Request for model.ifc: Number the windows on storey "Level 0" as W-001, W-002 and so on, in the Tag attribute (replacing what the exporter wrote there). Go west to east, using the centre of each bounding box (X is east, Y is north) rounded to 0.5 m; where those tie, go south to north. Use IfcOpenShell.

First a look at what the model holds.

```python
import ifcopenshell
import ifcopenshell.util.element
import ifcopenshell.util.placement

model = ifcopenshell.open("model.ifc")
print(model.schema)
storey = next(s for s in model.by_type("IfcBuildingStorey") if s.Name == "Level 0")
windows = [e for e in ifcopenshell.util.element.get_decomposition(storey) if e.is_a("IfcWindow")]
for e in sorted(windows, key=lambda e: e.id()):
    origin = ifcopenshell.util.placement.get_local_placement(e.ObjectPlacement)[:3, 3]
    print(e.id(), e.Tag, e.Name, origin.round(2) + 0.0, sep=" | ")
```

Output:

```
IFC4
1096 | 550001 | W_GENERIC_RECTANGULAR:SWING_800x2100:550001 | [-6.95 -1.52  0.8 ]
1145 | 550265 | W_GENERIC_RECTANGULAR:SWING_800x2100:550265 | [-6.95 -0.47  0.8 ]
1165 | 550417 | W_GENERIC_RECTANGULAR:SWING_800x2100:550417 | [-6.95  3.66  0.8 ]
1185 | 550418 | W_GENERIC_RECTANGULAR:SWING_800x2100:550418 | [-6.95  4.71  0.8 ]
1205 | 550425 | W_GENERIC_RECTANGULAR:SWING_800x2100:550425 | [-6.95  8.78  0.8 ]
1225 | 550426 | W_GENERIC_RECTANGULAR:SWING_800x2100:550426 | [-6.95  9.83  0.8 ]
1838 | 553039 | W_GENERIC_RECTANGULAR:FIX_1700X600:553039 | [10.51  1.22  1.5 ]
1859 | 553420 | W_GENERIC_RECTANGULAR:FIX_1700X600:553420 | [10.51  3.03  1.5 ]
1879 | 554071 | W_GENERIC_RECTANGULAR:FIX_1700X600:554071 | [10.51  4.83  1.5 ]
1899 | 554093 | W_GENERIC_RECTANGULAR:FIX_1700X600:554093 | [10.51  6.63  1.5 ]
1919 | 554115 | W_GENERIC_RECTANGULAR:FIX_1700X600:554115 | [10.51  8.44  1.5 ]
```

```python
import ifcopenshell
import ifcopenshell.geom
import ifcopenshell.util.element
import ifcopenshell.util.shape

model = ifcopenshell.open("model.ifc")
settings = ifcopenshell.geom.settings()
settings.set("use-world-coords", True)


def centre(element):
    shape = ifcopenshell.geom.create_shape(settings, element)
    return ifcopenshell.util.shape.get_bbox_centroid(shape.geometry)


storey = next(s for s in model.by_type("IfcBuildingStorey") if s.Name == "Level 0")
windows = [e for e in ifcopenshell.util.element.get_decomposition(storey) if e.is_a("IfcWindow")]

# Insertion points can sit at a corner or the storey origin, so sort by the geometry (in metres).
centres = {e: centre(e) for e in windows}
windows.sort(key=lambda e: (round(centres[e][0] / 0.5), centres[e][1]))

for i, e in enumerate(windows, start=1):
    number = f"W-0{i:02d}"
    e.Tag = number
    print(e.id(), number)

model.write("model_v2.ifc")
```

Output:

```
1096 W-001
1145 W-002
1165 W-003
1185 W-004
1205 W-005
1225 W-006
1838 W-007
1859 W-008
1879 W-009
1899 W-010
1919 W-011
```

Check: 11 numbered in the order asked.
